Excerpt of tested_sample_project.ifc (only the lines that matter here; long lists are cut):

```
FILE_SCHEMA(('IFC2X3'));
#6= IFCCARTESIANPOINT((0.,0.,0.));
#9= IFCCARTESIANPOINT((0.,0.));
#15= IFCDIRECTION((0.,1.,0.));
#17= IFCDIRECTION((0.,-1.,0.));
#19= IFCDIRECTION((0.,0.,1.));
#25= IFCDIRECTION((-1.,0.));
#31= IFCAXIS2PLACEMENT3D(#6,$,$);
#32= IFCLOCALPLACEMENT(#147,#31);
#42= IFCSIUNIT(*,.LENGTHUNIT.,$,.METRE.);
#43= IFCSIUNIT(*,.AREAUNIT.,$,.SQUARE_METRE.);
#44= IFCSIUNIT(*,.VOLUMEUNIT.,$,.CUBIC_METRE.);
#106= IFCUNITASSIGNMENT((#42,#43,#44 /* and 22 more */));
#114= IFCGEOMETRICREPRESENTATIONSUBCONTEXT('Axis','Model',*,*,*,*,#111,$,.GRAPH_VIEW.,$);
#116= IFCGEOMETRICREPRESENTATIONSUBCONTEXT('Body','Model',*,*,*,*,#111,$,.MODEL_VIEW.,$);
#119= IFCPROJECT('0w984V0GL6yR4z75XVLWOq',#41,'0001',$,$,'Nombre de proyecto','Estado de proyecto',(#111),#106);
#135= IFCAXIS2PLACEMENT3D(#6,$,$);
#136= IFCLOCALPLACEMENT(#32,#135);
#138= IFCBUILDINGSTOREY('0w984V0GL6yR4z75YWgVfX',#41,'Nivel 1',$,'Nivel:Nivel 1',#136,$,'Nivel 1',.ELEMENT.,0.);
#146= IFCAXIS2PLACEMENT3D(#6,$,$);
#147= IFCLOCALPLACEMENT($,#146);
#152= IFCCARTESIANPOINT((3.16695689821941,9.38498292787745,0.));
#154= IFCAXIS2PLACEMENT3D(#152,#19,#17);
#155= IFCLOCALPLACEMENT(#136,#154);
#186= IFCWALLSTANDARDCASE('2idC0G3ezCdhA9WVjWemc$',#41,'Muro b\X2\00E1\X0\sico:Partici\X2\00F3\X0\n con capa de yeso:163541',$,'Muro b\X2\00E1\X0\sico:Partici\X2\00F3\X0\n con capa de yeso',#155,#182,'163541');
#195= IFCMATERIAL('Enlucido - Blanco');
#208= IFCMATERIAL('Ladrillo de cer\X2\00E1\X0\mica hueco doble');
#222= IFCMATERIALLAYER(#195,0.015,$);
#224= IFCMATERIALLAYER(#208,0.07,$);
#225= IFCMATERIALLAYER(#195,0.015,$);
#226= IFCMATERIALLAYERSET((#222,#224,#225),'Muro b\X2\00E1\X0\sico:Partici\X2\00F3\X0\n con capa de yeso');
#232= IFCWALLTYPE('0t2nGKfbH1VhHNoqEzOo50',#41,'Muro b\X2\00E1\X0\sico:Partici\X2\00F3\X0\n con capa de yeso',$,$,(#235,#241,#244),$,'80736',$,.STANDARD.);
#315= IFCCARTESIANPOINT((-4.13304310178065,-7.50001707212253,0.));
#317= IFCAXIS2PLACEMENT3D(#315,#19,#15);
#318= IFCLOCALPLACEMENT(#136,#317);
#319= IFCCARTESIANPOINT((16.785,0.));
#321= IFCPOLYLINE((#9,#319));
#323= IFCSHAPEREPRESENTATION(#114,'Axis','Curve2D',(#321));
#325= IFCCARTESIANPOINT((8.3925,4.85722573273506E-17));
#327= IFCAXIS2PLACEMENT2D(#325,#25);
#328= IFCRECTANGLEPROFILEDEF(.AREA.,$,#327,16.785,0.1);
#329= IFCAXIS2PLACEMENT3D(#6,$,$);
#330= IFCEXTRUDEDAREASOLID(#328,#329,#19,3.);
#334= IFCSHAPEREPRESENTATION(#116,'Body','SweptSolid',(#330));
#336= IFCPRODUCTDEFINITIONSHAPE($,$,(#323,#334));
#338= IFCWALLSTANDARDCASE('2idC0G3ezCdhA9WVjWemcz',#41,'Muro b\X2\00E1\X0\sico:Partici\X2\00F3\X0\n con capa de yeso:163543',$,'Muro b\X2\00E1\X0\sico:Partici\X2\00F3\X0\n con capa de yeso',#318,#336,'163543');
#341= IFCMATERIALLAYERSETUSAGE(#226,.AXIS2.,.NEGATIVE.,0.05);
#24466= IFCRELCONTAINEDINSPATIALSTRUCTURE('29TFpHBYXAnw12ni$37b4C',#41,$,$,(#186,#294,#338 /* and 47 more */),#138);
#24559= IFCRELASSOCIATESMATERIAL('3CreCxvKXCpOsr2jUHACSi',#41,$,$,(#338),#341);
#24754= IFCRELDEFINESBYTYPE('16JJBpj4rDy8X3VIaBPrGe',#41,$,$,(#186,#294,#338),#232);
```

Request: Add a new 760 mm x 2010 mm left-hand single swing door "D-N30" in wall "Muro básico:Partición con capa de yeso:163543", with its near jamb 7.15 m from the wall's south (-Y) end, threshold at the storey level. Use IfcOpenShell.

```python
import numpy as np
import ifcopenshell
import ifcopenshell.api.feature
import ifcopenshell.api.geometry
import ifcopenshell.api.root
import ifcopenshell.api.spatial
import ifcopenshell.api.type
import ifcopenshell.geom
import ifcopenshell.util.element
import ifcopenshell.util.placement
import ifcopenshell.util.representation
import ifcopenshell.util.shape
import ifcopenshell.util.unit

model = ifcopenshell.open("tested_sample_project.ifc")
unit_scale = ifcopenshell.util.unit.calculate_unit_scale(model)
settings = ifcopenshell.geom.settings()


def volume(element):
    """Net volume in cubic metres, openings subtracted."""
    shape = ifcopenshell.geom.create_shape(settings, element)
    return ifcopenshell.util.shape.get_volume(shape.geometry)


wall = model.by_guid("2idC0G3ezCdhA9WVjWemcz")
storey = ifcopenshell.util.element.get_container(wall, ifc_class="IfcBuildingStorey")
context = ifcopenshell.util.representation.get_context(model, "Model", "Body", "MODEL_VIEW")
before = volume(wall)

width, height, from_end, sill = 0.76, 2.01, 7.15, 0.0  # metres

# The wall runs along its own X axis, and the end named is its -X end.
wall_shape = ifcopenshell.geom.create_shape(settings, wall)
x, y, z = ifcopenshell.util.shape.get_vertices(wall_shape.geometry).T
start = x.min() + from_end
face, thickness = float(y.min()), float(y.max() - y.min())
wall_matrix = ifcopenshell.util.placement.get_local_placement(wall.ObjectPlacement)
level = ifcopenshell.util.placement.get_local_placement(storey.ObjectPlacement)[2, 3]


def in_wall(x, y):
    """Placement at x, y metres in the wall's axes, at sill height."""
    matrix = wall_matrix.copy()
    matrix[:, 3] = wall_matrix @ np.array([x / unit_scale, y / unit_scale, 0.0, 1.0])
    matrix[2, 3] = level + sill / unit_scale
    return matrix


# Opening: a box that overshoots both wall faces by 50 mm.
opening = ifcopenshell.api.root.create_entity(model, ifc_class="IfcOpeningElement")
box = ifcopenshell.api.geometry.add_wall_representation(
    model, context=context, length=width, height=height, thickness=thickness + 0.1
)
ifcopenshell.api.geometry.assign_representation(model, product=opening, representation=box)
ifcopenshell.api.geometry.edit_object_placement(model, product=opening, matrix=in_wall(start, face - 0.05), is_si=False)
ifcopenshell.api.feature.add_feature(model, feature=opening, element=wall)

door = ifcopenshell.api.root.create_entity(model, ifc_class="IfcDoor", name="D-N30")
door.OverallWidth, door.OverallHeight = width / unit_scale, height / unit_scale
body = ifcopenshell.api.geometry.add_door_representation(
    model,
    context=context,
    overall_width=door.OverallWidth,
    overall_height=door.OverallHeight,
    operation_type="SINGLE_SWING_LEFT",
    lining_properties={"LiningDepth": thickness / unit_scale, "ThresholdDepth": thickness / unit_scale},
)
ifcopenshell.api.geometry.assign_representation(model, product=door, representation=body)
ifcopenshell.api.spatial.assign_container(model, products=[door], relating_structure=storey)
fills = ifcopenshell.api.feature.add_filling(model, opening=opening, element=door)
fills.OwnerHistory = door.OwnerHistory  # required in IFC2X3

# IFC2X3 keeps the operation on the door style.
style = ifcopenshell.api.root.create_entity(model, ifc_class="IfcDoorStyle", name="D-N30")
style.OperationType, style.ConstructionType = "SINGLE_SWING_LEFT", "NOTDEFINED"
style.ParameterTakesPrecedence = style.Sizeable = False
ifcopenshell.api.type.assign_type(model, related_objects=[door], relating_type=style)

# The lining spans the wall, so the door starts at the wall face.
ifcopenshell.api.geometry.edit_object_placement(model, product=door, matrix=in_wall(start, face), is_si=False)

after = volume(wall)

print(f"wall volume {before:.3f} -> {after:.3f} m3")

model.write("tested_sample_project_updated.ifc")
```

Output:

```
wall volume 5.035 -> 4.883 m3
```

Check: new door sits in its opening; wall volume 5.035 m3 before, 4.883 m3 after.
